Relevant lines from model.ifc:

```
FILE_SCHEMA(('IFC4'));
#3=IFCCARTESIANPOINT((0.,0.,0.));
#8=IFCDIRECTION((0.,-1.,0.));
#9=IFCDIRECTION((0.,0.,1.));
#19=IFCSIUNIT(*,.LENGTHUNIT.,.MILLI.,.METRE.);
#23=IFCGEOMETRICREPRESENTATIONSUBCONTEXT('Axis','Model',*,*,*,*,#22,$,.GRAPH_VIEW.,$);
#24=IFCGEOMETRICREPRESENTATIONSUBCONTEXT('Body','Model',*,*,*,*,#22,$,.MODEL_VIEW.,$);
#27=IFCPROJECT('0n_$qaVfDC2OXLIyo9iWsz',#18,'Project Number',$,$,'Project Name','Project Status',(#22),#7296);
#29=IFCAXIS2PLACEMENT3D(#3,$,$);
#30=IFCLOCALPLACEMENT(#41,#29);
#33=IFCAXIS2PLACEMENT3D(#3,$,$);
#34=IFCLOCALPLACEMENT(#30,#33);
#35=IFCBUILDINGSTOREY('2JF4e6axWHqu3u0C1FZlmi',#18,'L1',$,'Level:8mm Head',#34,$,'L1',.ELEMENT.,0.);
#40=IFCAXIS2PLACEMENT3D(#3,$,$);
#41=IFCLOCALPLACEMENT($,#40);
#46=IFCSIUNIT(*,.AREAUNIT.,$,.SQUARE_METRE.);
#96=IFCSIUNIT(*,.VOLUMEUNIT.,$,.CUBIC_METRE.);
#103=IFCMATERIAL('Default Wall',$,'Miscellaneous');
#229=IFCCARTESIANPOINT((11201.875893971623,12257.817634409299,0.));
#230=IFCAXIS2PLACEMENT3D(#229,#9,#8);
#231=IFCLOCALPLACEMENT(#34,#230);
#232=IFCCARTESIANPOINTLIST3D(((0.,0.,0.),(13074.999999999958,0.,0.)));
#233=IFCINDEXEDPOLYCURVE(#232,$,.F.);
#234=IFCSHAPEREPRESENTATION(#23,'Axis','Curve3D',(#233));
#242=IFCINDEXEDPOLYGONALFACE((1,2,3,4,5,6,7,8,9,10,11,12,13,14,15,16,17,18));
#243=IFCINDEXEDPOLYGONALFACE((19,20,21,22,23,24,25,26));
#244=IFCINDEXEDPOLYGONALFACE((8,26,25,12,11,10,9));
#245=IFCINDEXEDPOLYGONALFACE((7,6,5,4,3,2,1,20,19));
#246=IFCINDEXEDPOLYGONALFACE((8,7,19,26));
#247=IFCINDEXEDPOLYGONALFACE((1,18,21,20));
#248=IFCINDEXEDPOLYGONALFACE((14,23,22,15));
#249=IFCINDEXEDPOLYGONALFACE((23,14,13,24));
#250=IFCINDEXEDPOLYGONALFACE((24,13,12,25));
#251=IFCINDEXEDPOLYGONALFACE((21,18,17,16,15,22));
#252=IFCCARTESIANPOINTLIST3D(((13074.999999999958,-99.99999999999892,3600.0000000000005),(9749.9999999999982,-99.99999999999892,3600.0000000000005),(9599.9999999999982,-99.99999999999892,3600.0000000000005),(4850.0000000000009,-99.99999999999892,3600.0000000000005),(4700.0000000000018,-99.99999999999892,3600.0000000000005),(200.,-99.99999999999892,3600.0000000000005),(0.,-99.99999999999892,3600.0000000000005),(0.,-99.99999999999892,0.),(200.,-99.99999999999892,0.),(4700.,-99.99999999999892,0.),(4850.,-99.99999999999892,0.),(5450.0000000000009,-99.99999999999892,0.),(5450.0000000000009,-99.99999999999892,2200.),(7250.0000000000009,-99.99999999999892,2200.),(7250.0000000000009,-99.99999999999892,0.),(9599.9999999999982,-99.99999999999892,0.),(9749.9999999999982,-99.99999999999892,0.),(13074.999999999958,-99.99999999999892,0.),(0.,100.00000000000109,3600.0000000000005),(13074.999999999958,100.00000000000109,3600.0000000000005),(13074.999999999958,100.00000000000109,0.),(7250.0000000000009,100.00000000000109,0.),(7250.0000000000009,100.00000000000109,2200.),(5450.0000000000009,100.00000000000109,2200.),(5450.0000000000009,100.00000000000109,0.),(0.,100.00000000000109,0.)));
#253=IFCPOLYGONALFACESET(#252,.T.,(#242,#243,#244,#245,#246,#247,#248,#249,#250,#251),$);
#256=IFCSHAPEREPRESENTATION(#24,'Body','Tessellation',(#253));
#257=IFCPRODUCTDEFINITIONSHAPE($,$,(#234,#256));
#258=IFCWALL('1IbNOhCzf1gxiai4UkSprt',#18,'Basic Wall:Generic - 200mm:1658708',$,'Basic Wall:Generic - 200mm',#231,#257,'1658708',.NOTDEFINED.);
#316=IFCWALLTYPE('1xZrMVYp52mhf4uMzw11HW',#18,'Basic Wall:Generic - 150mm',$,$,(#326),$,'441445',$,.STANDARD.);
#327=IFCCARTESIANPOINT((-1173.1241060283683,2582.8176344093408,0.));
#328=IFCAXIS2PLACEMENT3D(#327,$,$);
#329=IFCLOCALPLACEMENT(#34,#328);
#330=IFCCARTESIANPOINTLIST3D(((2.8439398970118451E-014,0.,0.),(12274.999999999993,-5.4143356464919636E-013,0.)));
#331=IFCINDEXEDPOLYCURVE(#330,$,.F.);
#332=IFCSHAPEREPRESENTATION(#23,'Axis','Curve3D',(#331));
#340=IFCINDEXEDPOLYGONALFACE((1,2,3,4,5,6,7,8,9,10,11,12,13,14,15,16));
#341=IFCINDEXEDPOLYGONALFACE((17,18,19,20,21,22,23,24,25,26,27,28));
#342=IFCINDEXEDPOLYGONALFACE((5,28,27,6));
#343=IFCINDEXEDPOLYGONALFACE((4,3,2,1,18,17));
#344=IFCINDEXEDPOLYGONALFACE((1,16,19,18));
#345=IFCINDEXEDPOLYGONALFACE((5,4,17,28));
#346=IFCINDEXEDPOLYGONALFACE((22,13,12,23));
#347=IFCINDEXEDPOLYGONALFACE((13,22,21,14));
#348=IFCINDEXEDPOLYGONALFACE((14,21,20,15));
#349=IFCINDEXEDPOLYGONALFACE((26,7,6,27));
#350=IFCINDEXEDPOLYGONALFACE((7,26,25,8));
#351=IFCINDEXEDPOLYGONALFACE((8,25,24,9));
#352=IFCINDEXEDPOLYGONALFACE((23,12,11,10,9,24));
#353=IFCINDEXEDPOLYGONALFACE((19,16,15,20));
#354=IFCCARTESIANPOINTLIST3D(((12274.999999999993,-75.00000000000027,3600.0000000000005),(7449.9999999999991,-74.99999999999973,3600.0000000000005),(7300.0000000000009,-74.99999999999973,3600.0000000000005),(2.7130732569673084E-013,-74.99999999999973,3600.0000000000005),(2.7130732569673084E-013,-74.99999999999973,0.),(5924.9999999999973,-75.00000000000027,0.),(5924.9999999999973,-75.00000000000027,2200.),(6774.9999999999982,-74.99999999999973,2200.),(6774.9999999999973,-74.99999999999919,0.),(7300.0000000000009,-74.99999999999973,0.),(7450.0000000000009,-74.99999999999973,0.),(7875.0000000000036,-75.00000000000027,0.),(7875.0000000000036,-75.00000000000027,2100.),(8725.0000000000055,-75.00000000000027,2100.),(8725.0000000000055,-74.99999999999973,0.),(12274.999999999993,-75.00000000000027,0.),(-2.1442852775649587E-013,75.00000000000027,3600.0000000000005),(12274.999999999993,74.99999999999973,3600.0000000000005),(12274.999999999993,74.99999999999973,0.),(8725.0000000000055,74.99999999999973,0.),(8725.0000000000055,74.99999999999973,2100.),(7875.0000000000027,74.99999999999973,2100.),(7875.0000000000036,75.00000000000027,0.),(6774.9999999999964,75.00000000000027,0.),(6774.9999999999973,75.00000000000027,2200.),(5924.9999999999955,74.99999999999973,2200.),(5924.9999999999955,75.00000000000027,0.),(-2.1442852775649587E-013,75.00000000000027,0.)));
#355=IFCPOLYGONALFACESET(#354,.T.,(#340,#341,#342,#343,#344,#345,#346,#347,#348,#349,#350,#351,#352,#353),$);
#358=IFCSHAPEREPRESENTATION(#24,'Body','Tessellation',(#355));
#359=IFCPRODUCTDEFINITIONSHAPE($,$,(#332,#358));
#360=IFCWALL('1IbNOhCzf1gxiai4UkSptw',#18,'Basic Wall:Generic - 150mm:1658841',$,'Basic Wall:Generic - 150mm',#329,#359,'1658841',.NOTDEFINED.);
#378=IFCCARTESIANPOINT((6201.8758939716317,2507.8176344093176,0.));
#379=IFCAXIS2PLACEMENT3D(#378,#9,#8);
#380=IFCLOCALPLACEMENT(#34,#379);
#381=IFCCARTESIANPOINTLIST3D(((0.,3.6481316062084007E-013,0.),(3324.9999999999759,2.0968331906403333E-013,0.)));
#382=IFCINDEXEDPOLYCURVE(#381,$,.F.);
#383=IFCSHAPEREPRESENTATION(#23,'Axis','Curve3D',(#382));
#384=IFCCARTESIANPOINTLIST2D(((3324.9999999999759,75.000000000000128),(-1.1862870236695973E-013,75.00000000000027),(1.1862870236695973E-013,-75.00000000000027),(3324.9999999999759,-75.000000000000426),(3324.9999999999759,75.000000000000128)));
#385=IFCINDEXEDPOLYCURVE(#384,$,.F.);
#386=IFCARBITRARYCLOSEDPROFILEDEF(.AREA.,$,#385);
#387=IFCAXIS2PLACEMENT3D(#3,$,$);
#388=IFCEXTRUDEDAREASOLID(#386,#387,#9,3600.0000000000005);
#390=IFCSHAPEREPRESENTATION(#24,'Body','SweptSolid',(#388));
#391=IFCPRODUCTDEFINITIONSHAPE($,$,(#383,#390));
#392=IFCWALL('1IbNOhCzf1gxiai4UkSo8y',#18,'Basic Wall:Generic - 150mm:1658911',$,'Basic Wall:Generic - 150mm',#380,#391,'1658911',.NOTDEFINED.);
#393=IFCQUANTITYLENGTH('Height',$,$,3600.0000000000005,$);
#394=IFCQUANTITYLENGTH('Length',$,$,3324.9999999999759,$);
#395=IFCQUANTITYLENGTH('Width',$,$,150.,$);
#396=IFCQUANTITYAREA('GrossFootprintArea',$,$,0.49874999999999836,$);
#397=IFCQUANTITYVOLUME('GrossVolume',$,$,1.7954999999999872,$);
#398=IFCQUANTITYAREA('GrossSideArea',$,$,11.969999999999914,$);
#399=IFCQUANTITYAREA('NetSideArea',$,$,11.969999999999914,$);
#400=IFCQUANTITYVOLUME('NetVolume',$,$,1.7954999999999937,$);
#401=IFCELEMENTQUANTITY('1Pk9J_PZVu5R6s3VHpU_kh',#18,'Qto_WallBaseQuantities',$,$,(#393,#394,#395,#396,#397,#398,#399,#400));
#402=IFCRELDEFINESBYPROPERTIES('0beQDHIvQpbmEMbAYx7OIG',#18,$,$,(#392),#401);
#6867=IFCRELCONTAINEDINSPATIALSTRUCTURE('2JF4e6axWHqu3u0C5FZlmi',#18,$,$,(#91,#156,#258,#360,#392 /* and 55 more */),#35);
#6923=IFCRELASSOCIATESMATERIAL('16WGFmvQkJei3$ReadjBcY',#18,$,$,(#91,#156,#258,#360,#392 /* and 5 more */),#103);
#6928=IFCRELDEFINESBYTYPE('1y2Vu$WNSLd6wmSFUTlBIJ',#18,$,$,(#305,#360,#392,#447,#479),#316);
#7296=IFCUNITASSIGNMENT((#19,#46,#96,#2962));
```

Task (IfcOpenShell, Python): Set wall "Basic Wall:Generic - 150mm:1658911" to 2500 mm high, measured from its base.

```python
import ifcopenshell
import ifcopenshell.api.pset
import ifcopenshell.geom
import ifcopenshell.util.element
import ifcopenshell.util.representation
import ifcopenshell.util.shape
import ifcopenshell.util.unit

model = ifcopenshell.open("model.ifc")
unit_scale = ifcopenshell.util.unit.calculate_unit_scale(model)
area_scale = ifcopenshell.util.unit.calculate_unit_scale(model, "AREAUNIT")
volume_scale = ifcopenshell.util.unit.calculate_unit_scale(model, "VOLUMEUNIT")
settings = ifcopenshell.geom.settings()


def volume(element):
    """Net volume in cubic metres, openings subtracted."""
    shape = ifcopenshell.geom.create_shape(settings, element)
    return ifcopenshell.util.shape.get_volume(shape.geometry)


wall = model.by_guid("1IbNOhCzf1gxiai4UkSo8y")
before = volume(wall)

body = ifcopenshell.util.representation.get_representation(wall, "Model", "Body")
solid = body.Items[0]
old_height = solid.Depth
solid.Depth = 2500.0
after = volume(wall)
thickness = 0.15  # wall thickness in metres

# Update the stored height, areas and volumes.
qto = model.by_id(ifcopenshell.util.element.get_pset(wall, "Qto_WallBaseQuantities", should_inherit=False)["id"])
ifcopenshell.api.pset.edit_qto(model, qto=qto, properties={
    "Height": solid.Depth,
    "GrossVolume": ifcopenshell.util.element.get_pset(wall, "Qto_WallBaseQuantities", "GrossVolume") * solid.Depth / old_height,
    "GrossSideArea": ifcopenshell.util.element.get_pset(wall, "Qto_WallBaseQuantities", "GrossSideArea") * solid.Depth / old_height,
    "NetSideArea": after / thickness / area_scale,
    "NetVolume": after / volume_scale,
})

print(f"height {old_height:g} -> {solid.Depth:g}, volume {before:.3f} -> {after:.3f} m3")

model.write("model_rev.ifc")
```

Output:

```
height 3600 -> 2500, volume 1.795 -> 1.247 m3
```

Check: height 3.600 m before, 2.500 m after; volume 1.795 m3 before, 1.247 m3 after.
